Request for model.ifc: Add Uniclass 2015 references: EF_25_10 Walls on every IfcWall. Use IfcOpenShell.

First a look at what the model holds.

```python
import ifcopenshell

model = ifcopenshell.open("model.ifc")
print(model.schema)
print("classifications:", [c.Name for c in model.by_type("IfcClassification")])
for ifc_class in ("IfcDoor", "IfcRoof", "IfcStair", "IfcWall", "IfcWindow"):
    print(ifc_class, len(model.by_type(ifc_class)))
```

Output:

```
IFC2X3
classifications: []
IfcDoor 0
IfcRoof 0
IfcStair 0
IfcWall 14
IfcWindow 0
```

```python
import ifcopenshell
import ifcopenshell.api.classification

model = ifcopenshell.open("model.ifc")

# IFC2X3 requires Source and Edition and has no link from the project to the system.
system = model.create_entity("IfcClassification", Source="NBS", Edition="2015", Name="Uniclass 2015")

codes = {
    "IfcWall": ("EF_25_10", "Walls"),
}
for ifc_class, (code, name) in codes.items():
    products = model.by_type(ifc_class)
    ifcopenshell.api.classification.add_reference(
        model, products=products, classification=system, identification=code, name=name
    )
    print(code, len(products))

model.write("model_updated.ifc")
```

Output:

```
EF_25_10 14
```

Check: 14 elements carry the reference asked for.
